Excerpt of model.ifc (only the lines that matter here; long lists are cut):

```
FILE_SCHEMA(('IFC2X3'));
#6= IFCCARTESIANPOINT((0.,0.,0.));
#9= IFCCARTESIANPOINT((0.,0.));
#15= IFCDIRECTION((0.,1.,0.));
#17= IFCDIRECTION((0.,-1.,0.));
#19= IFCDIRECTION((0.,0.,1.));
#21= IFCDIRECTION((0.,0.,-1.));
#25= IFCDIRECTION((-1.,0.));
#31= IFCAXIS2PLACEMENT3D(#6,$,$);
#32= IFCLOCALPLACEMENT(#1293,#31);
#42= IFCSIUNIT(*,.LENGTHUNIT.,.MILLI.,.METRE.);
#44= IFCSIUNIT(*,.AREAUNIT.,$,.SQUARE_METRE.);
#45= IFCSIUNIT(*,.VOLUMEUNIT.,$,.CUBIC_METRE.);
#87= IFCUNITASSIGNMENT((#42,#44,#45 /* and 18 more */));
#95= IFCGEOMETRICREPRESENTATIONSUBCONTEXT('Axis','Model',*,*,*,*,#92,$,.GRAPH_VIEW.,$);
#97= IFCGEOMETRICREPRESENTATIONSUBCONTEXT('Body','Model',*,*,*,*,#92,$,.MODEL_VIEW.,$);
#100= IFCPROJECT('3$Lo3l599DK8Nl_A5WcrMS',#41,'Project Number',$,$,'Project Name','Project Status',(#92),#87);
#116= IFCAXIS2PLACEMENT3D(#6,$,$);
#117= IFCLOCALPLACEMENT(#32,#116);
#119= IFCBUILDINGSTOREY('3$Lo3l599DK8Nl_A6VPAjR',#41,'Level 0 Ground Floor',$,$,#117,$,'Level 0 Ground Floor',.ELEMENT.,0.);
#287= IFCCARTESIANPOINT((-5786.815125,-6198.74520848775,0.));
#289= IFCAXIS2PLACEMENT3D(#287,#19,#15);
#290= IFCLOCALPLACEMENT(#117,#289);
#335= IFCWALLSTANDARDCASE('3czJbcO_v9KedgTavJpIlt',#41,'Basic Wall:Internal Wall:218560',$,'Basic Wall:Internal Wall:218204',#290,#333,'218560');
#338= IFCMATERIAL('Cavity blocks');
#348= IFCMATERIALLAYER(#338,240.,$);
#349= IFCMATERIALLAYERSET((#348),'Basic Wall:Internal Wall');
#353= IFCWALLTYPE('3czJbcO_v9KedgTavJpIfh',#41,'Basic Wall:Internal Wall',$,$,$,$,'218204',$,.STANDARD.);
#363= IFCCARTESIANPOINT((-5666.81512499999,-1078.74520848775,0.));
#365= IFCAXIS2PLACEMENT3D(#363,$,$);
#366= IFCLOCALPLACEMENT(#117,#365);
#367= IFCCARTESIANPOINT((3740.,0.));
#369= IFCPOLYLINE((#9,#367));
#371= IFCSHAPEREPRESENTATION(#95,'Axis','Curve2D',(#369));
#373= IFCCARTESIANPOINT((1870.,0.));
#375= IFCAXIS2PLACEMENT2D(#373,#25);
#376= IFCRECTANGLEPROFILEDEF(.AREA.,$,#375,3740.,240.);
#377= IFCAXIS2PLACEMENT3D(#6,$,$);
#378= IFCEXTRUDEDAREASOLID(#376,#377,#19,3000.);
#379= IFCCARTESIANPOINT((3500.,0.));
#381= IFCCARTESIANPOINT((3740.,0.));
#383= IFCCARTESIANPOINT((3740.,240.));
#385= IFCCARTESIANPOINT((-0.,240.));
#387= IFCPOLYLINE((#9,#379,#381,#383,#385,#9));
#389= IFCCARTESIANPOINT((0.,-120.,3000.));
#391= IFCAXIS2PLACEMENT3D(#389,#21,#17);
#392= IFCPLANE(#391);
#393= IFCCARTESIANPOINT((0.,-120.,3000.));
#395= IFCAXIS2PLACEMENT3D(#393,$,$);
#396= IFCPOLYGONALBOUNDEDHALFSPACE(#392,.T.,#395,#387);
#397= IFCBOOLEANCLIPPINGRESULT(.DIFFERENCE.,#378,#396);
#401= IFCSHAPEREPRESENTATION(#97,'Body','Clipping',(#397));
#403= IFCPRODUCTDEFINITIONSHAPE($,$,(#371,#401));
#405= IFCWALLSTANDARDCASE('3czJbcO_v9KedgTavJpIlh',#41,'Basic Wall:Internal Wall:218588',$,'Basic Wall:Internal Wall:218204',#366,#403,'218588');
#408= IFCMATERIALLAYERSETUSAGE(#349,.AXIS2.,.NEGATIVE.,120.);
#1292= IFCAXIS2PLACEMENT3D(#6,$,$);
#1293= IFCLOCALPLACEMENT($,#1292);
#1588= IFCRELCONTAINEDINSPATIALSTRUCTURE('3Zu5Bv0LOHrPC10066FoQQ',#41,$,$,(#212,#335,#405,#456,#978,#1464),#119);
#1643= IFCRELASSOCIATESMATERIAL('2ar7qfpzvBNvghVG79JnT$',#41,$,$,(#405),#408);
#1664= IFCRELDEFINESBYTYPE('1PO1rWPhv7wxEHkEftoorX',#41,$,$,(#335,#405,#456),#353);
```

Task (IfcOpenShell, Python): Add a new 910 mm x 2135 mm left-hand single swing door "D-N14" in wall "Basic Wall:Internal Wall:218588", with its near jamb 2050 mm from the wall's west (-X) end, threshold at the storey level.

```python
import numpy as np
import ifcopenshell
import ifcopenshell.api.feature
import ifcopenshell.api.geometry
import ifcopenshell.api.root
import ifcopenshell.api.spatial
import ifcopenshell.api.type
import ifcopenshell.geom
import ifcopenshell.util.element
import ifcopenshell.util.placement
import ifcopenshell.util.representation
import ifcopenshell.util.shape
import ifcopenshell.util.unit

model = ifcopenshell.open("model.ifc")
unit_scale = ifcopenshell.util.unit.calculate_unit_scale(model)
settings = ifcopenshell.geom.settings()


def volume(element):
    """Net volume in cubic metres, openings subtracted."""
    shape = ifcopenshell.geom.create_shape(settings, element)
    return ifcopenshell.util.shape.get_volume(shape.geometry)


wall = model.by_id(405)
storey = ifcopenshell.util.element.get_container(wall, ifc_class="IfcBuildingStorey")
context = ifcopenshell.util.representation.get_context(model, "Model", "Body", "MODEL_VIEW")
before = volume(wall)

width, height, from_end, sill = 0.91, 2.135, 2.05, 0.0  # metres

# The wall runs along its own X axis, and the end named is its -X end.
wall_shape = ifcopenshell.geom.create_shape(settings, wall)
x, y, z = ifcopenshell.util.shape.get_vertices(wall_shape.geometry).T
start = x.min() + from_end
face, thickness = float(y.min()), float(y.max() - y.min())
wall_matrix = ifcopenshell.util.placement.get_local_placement(wall.ObjectPlacement)
level = ifcopenshell.util.placement.get_local_placement(storey.ObjectPlacement)[2, 3]


def in_wall(x, y):
    """Placement at x, y metres in the wall's axes, at sill height."""
    matrix = wall_matrix.copy()
    matrix[:, 3] = wall_matrix @ np.array([x / unit_scale, y / unit_scale, 0.0, 1.0])
    matrix[2, 3] = level + sill / unit_scale
    return matrix


# Opening: a box that overshoots both wall faces by 50 mm.
opening = ifcopenshell.api.root.create_entity(model, ifc_class="IfcOpeningElement")
box = ifcopenshell.api.geometry.add_wall_representation(
    model, context=context, length=width, height=height, thickness=thickness + 0.1
)
ifcopenshell.api.geometry.assign_representation(model, product=opening, representation=box)
ifcopenshell.api.geometry.edit_object_placement(model, product=opening, matrix=in_wall(start, face - 0.05), is_si=False)
ifcopenshell.api.feature.add_feature(model, feature=opening, element=wall)

door = ifcopenshell.api.root.create_entity(model, ifc_class="IfcDoor", name="D-N14")
door.OverallWidth, door.OverallHeight = width / unit_scale, height / unit_scale
body = ifcopenshell.api.geometry.add_door_representation(
    model,
    context=context,
    overall_width=door.OverallWidth,
    overall_height=door.OverallHeight,
    operation_type="SINGLE_SWING_LEFT",
    lining_properties={"LiningDepth": thickness / unit_scale, "ThresholdDepth": thickness / unit_scale},
)
ifcopenshell.api.geometry.assign_representation(model, product=door, representation=body)
ifcopenshell.api.spatial.assign_container(model, products=[door], relating_structure=storey)
fills = ifcopenshell.api.feature.add_filling(model, opening=opening, element=door)
fills.OwnerHistory = door.OwnerHistory  # required in IFC2X3

# IFC2X3 keeps the operation on the door style.
style = ifcopenshell.api.root.create_entity(model, ifc_class="IfcDoorStyle", name="D-N14")
style.OperationType, style.ConstructionType = "SINGLE_SWING_LEFT", "NOTDEFINED"
style.ParameterTakesPrecedence = style.Sizeable = False
ifcopenshell.api.type.assign_type(model, related_objects=[door], relating_type=style)

# The lining spans the wall, so the door starts at the wall face.
ifcopenshell.api.geometry.edit_object_placement(model, product=door, matrix=in_wall(start, face), is_si=False)

after = volume(wall)

print(f"wall volume {before:.3f} -> {after:.3f} m3")

model.write("model_edited.ifc")
```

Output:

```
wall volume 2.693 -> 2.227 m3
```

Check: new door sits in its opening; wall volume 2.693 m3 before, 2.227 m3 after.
